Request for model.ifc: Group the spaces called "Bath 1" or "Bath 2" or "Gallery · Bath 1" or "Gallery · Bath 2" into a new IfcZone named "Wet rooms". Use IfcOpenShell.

First a look at what the model holds.

```python
import ifcopenshell

model = ifcopenshell.open("model.ifc")
print(model.schema)
seen = {}
for space in model.by_type("IfcSpace"):
    seen[space.Name] = seen.get(space.Name, 0) + 1
for name, count in sorted(seen.items(), key=str):
    print(count, "x", name)
print("zones:", [z.Name for z in model.by_type("IfcZone")][:20])
```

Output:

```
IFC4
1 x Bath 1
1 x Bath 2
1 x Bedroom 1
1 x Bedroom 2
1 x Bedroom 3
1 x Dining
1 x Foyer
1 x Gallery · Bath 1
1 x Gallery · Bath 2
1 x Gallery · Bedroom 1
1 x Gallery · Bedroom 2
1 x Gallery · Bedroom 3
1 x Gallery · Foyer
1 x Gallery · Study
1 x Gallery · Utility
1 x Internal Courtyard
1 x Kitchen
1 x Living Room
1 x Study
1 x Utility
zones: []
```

```python
import ifcopenshell
import ifcopenshell.api.group
import ifcopenshell.api.root

model = ifcopenshell.open("model.ifc")

names = {"Bath 1", "Bath 2", "Gallery · Bath 1", "Gallery · Bath 2"}
spaces = [s for s in model.by_type("IfcSpace") if s.Name in names]

zone = ifcopenshell.api.root.create_entity(model, ifc_class="IfcZone", name="Wet rooms")
ifcopenshell.api.group.assign_group(model, products=spaces, group=zone)
print(len(spaces), "spaces in", zone.Name)

model.write("model_edited.ifc")
```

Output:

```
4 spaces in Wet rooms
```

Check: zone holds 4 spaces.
